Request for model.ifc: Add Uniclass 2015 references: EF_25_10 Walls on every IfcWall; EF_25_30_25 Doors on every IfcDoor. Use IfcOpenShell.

First a look at what the model holds.

```python
import ifcopenshell

model = ifcopenshell.open("model.ifc")
print(model.schema)
print("classifications:", [c.Name for c in model.by_type("IfcClassification")])
for ifc_class in ("IfcDoor", "IfcRoof", "IfcStair", "IfcWall", "IfcWindow"):
    print(ifc_class, len(model.by_type(ifc_class)))
```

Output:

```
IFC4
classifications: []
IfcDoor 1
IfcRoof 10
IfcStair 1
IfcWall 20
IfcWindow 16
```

```python
import ifcopenshell
import ifcopenshell.api.classification

model = ifcopenshell.open("model.ifc")

system = ifcopenshell.api.classification.add_classification(model, classification="Uniclass 2015")

codes = {
    "IfcWall": ("EF_25_10", "Walls"),
    "IfcDoor": ("EF_25_30_25", "Doors"),
}
for ifc_class, (code, name) in codes.items():
    products = model.by_type(ifc_class)
    ifcopenshell.api.classification.add_reference(
        model, products=products, classification=system, identification=code, name=name
    )
    print(code, len(products))

model.write("model_v2.ifc")
```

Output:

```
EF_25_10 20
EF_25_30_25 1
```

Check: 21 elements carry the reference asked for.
